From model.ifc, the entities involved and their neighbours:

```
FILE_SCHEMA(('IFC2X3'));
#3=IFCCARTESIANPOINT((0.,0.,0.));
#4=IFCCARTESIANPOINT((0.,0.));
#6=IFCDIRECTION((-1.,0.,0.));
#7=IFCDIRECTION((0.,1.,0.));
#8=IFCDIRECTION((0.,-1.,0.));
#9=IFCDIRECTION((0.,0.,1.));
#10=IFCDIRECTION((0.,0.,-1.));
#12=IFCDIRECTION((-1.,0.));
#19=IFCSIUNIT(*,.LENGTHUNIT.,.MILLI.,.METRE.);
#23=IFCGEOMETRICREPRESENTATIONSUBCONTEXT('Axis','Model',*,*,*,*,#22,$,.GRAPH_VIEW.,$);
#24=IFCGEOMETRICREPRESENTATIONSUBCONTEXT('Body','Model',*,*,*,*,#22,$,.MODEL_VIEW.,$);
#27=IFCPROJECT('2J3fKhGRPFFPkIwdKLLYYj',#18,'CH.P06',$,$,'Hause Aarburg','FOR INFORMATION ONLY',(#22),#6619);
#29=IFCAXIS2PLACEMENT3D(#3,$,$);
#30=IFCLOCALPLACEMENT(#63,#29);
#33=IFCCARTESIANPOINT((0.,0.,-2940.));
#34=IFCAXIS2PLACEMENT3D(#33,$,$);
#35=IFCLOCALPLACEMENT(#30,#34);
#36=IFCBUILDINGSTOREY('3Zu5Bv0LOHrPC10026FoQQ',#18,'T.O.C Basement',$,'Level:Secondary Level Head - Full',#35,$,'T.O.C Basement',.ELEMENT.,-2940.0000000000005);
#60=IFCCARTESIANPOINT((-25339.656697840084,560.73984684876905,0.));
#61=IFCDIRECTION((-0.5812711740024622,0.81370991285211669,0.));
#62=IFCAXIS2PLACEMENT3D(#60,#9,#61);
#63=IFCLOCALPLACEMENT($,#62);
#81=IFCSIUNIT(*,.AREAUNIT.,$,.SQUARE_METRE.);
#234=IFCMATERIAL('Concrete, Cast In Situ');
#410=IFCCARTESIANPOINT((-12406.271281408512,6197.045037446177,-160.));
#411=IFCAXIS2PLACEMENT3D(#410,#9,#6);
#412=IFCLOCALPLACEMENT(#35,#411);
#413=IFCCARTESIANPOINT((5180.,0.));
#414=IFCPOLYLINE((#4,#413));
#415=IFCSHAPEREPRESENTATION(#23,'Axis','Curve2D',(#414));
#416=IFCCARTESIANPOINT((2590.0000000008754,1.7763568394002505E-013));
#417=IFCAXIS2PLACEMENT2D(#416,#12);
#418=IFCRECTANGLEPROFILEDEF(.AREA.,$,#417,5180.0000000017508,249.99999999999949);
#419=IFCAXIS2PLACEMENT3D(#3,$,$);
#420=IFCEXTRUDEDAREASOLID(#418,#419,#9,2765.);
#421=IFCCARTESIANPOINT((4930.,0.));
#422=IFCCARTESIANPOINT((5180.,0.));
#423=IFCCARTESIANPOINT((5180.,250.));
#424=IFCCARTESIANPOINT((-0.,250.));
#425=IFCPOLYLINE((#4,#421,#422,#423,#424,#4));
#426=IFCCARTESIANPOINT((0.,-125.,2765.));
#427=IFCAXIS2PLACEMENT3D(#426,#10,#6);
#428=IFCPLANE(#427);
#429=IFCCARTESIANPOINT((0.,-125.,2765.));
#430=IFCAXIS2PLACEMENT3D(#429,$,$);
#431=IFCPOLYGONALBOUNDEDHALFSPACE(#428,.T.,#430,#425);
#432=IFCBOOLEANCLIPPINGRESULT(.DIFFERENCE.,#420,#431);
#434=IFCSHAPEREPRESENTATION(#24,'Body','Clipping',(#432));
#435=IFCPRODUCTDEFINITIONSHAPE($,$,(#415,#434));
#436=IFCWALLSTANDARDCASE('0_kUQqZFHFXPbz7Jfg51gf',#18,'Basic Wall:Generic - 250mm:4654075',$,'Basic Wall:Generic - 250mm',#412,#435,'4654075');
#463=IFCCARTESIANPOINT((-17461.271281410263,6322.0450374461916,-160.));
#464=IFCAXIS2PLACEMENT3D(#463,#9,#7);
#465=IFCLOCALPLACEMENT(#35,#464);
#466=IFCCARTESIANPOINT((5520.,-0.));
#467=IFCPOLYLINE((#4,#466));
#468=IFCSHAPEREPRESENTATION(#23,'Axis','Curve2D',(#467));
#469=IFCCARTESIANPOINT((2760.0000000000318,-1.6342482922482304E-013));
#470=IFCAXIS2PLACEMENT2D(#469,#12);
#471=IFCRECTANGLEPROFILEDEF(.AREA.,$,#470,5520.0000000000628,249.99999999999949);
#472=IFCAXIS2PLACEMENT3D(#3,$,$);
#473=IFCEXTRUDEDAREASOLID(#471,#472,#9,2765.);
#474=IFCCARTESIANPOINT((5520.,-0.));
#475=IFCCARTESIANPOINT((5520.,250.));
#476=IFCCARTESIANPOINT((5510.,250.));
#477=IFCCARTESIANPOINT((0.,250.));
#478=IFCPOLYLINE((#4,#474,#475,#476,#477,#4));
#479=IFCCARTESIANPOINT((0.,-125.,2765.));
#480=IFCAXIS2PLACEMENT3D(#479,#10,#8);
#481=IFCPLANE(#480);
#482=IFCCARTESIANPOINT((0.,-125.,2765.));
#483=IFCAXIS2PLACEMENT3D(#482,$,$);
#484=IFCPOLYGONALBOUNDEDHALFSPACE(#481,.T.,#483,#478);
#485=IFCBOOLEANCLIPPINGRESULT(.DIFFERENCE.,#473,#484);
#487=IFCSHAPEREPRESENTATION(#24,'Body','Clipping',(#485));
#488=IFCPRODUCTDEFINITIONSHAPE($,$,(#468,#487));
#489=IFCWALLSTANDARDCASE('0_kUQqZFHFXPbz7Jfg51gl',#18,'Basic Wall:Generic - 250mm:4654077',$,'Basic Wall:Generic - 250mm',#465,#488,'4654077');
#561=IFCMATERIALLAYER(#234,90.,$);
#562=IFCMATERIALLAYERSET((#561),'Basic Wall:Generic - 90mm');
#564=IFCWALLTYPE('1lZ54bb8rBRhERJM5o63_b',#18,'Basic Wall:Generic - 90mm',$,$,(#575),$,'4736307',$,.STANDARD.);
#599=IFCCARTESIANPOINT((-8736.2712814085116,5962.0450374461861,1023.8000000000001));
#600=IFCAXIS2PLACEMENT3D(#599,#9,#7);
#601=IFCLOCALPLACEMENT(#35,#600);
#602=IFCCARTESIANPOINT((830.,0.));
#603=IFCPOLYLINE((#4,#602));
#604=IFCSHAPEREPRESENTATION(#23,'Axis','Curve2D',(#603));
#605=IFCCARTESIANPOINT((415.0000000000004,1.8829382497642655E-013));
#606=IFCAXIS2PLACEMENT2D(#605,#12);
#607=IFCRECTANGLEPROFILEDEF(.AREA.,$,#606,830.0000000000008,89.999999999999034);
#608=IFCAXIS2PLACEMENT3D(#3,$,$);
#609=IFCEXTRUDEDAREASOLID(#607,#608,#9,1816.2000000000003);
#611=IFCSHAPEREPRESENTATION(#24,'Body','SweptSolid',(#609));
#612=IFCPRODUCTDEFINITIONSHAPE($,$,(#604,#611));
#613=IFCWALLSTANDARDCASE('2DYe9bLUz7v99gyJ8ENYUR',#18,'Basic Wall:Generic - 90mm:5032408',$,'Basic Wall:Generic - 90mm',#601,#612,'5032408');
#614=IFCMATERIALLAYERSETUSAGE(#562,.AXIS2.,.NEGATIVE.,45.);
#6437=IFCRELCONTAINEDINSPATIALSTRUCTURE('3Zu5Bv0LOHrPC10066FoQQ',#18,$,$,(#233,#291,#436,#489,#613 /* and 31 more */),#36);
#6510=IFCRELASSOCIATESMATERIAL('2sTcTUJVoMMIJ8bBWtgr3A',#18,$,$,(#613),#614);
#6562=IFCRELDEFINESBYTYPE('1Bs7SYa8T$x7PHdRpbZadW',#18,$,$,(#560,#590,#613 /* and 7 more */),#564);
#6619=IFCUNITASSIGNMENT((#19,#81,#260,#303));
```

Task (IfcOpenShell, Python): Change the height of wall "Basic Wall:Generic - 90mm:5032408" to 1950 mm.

```python
import ifcopenshell
import ifcopenshell.geom
import ifcopenshell.util.representation
import ifcopenshell.util.shape
import ifcopenshell.util.unit

model = ifcopenshell.open("model.ifc")
unit_scale = ifcopenshell.util.unit.calculate_unit_scale(model)
settings = ifcopenshell.geom.settings()


def volume(element):
    """Net volume in cubic metres, openings subtracted."""
    shape = ifcopenshell.geom.create_shape(settings, element)
    return ifcopenshell.util.shape.get_volume(shape.geometry)


wall = model.by_id(613)
before = volume(wall)

body = ifcopenshell.util.representation.get_representation(wall, "Model", "Body")
solid = body.Items[0]
old_height = solid.Depth
solid.Depth = 1.95 / unit_scale
after = volume(wall)

print(f"height {old_height:g} -> {solid.Depth:g}, volume {before:.3f} -> {after:.3f} m3")

model.write("model_v2.ifc")
```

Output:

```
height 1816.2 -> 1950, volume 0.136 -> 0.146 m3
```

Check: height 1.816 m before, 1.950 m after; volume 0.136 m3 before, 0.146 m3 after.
